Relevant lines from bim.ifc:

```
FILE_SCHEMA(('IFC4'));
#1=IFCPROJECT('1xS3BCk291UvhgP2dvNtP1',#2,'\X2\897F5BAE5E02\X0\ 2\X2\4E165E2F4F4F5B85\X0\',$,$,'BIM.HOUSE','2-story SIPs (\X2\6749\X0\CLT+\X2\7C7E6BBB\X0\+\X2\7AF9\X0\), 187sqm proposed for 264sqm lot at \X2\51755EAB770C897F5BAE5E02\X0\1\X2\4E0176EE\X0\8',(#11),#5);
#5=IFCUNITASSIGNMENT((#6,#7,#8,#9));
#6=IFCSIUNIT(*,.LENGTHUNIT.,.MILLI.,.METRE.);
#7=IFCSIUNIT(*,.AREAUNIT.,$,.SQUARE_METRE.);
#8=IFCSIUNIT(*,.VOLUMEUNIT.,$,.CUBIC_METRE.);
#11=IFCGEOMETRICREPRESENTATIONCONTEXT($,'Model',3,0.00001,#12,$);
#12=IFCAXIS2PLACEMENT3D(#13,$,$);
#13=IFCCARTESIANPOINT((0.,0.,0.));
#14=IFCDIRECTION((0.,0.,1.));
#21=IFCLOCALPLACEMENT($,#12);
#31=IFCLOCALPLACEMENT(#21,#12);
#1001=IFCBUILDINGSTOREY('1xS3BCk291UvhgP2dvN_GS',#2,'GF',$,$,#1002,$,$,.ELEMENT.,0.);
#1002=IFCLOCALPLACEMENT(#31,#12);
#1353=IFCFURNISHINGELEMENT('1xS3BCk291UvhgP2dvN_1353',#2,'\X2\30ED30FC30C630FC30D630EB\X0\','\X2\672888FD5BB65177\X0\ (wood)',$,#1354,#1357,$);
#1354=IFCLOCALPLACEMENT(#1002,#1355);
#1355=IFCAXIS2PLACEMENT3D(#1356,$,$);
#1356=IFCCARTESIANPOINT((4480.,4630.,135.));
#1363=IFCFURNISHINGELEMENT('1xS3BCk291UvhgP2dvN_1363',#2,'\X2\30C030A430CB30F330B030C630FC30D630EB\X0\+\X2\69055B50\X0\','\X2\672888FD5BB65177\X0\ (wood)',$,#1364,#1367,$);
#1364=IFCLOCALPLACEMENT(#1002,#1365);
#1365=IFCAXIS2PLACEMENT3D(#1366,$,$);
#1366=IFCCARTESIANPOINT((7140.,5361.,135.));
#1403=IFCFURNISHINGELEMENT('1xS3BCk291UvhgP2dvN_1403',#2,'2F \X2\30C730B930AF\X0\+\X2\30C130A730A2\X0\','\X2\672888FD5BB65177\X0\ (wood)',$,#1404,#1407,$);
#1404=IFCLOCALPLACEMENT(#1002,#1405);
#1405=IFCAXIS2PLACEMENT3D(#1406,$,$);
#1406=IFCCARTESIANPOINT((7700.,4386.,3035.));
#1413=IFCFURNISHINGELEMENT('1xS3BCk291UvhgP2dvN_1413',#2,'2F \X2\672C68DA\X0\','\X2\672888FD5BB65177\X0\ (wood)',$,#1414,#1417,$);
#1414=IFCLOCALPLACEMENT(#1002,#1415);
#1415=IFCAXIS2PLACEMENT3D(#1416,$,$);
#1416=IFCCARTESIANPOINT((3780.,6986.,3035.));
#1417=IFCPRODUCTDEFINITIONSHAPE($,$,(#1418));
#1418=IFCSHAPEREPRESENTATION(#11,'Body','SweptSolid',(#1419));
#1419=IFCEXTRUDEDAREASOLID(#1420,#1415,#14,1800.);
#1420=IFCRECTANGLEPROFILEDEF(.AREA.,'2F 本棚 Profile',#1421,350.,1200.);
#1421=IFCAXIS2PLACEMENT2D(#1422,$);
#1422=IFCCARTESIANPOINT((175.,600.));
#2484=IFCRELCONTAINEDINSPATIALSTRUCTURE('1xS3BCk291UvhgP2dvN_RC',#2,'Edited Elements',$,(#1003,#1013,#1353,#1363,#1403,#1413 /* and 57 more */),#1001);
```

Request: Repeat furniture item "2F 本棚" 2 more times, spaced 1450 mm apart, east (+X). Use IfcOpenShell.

```python
import numpy as np
import ifcopenshell
import ifcopenshell.api.geometry
import ifcopenshell.api.root
import ifcopenshell.util.element
import ifcopenshell.util.placement

model = ifcopenshell.open("bim.ifc")


def reuse_history(source, copy):
    """copy_class also copies each property set's owner history, people and application; keep the originals."""
    for rel in copy.IsDefinedBy:
        if rel.is_a("IfcRelDefinesByProperties") and (history := rel.RelatingPropertyDefinition.OwnerHistory):
            rel.RelatingPropertyDefinition.OwnerHistory = source.OwnerHistory
            ifcopenshell.util.element.remove_deep2(model, history)


source = model.by_id(1413)
base = ifcopenshell.util.placement.get_local_placement(source.ObjectPlacement)
step = np.array([1.0, 0.0, 0.0]) * 1450.0

for i in range(1, 3):
    copy = ifcopenshell.api.root.copy_class(model, product=source)
    copy.Representation = ifcopenshell.util.element.copy_deep(
        model, source.Representation, exclude=["IfcGeometricRepresentationContext", "IfcRepresentationMap"]
    )
    reuse_history(source, copy)
    matrix = base.copy()
    matrix[:3, 3] += i * step
    print("added at", matrix[:3, 3].round(3) + 0.0)
    ifcopenshell.api.geometry.edit_object_placement(model, product=copy, matrix=matrix, is_si=False)

model.write("bim_updated.ifc")
```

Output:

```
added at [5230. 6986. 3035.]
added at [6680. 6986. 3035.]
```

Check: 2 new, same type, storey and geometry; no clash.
